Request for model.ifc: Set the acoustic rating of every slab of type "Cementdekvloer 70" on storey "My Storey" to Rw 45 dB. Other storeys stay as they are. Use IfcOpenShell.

First a look at what the model holds.

```python
import ifcopenshell
import ifcopenshell.util.element

model = ifcopenshell.open("model.ifc")
print(model.schema)
storey = next(s for s in model.by_type("IfcBuildingStorey") if s.Name == "My Storey")
slabs = [e for e in ifcopenshell.util.element.get_decomposition(storey) if e.is_a("IfcSlab")]
seen = {}
for e in slabs:
    element_type = ifcopenshell.util.element.get_type(e)
    key = (element_type.Name if element_type != e and element_type else None, ifcopenshell.util.element.get_pset(e, "Pset_SlabCommon", "AcousticRating"))
    seen[key] = seen.get(key, 0) + 1
for (name, value), count in sorted(seen.items(), key=str):
    print(count, "x", name, "|", value)
```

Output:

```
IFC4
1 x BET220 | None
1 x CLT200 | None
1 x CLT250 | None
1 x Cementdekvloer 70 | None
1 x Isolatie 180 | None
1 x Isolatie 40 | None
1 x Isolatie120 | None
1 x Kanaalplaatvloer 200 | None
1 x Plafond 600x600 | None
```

```python
import ifcopenshell
import ifcopenshell.api.pset
import ifcopenshell.util.element

model = ifcopenshell.open("model.ifc")

storey = next(s for s in model.by_type("IfcBuildingStorey") if s.Name == "My Storey")
slabs = [e for e in ifcopenshell.util.element.get_decomposition(storey) if e.is_a("IfcSlab")]

count = 0
for e in slabs:
    element_type = ifcopenshell.util.element.get_type(e)
    if element_type in (None, e) or element_type.Name != "Cementdekvloer 70":
        continue
    # add_pset returns the element's existing set when there is one.
    pset = ifcopenshell.api.pset.add_pset(model, product=e, name="Pset_SlabCommon")
    ifcopenshell.api.pset.edit_pset(model, pset=pset, properties={"AcousticRating": "Rw 45 dB"})
    count += 1

print(count, "slabs updated")

model.write("model_updated.ifc")
```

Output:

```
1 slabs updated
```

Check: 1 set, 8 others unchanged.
